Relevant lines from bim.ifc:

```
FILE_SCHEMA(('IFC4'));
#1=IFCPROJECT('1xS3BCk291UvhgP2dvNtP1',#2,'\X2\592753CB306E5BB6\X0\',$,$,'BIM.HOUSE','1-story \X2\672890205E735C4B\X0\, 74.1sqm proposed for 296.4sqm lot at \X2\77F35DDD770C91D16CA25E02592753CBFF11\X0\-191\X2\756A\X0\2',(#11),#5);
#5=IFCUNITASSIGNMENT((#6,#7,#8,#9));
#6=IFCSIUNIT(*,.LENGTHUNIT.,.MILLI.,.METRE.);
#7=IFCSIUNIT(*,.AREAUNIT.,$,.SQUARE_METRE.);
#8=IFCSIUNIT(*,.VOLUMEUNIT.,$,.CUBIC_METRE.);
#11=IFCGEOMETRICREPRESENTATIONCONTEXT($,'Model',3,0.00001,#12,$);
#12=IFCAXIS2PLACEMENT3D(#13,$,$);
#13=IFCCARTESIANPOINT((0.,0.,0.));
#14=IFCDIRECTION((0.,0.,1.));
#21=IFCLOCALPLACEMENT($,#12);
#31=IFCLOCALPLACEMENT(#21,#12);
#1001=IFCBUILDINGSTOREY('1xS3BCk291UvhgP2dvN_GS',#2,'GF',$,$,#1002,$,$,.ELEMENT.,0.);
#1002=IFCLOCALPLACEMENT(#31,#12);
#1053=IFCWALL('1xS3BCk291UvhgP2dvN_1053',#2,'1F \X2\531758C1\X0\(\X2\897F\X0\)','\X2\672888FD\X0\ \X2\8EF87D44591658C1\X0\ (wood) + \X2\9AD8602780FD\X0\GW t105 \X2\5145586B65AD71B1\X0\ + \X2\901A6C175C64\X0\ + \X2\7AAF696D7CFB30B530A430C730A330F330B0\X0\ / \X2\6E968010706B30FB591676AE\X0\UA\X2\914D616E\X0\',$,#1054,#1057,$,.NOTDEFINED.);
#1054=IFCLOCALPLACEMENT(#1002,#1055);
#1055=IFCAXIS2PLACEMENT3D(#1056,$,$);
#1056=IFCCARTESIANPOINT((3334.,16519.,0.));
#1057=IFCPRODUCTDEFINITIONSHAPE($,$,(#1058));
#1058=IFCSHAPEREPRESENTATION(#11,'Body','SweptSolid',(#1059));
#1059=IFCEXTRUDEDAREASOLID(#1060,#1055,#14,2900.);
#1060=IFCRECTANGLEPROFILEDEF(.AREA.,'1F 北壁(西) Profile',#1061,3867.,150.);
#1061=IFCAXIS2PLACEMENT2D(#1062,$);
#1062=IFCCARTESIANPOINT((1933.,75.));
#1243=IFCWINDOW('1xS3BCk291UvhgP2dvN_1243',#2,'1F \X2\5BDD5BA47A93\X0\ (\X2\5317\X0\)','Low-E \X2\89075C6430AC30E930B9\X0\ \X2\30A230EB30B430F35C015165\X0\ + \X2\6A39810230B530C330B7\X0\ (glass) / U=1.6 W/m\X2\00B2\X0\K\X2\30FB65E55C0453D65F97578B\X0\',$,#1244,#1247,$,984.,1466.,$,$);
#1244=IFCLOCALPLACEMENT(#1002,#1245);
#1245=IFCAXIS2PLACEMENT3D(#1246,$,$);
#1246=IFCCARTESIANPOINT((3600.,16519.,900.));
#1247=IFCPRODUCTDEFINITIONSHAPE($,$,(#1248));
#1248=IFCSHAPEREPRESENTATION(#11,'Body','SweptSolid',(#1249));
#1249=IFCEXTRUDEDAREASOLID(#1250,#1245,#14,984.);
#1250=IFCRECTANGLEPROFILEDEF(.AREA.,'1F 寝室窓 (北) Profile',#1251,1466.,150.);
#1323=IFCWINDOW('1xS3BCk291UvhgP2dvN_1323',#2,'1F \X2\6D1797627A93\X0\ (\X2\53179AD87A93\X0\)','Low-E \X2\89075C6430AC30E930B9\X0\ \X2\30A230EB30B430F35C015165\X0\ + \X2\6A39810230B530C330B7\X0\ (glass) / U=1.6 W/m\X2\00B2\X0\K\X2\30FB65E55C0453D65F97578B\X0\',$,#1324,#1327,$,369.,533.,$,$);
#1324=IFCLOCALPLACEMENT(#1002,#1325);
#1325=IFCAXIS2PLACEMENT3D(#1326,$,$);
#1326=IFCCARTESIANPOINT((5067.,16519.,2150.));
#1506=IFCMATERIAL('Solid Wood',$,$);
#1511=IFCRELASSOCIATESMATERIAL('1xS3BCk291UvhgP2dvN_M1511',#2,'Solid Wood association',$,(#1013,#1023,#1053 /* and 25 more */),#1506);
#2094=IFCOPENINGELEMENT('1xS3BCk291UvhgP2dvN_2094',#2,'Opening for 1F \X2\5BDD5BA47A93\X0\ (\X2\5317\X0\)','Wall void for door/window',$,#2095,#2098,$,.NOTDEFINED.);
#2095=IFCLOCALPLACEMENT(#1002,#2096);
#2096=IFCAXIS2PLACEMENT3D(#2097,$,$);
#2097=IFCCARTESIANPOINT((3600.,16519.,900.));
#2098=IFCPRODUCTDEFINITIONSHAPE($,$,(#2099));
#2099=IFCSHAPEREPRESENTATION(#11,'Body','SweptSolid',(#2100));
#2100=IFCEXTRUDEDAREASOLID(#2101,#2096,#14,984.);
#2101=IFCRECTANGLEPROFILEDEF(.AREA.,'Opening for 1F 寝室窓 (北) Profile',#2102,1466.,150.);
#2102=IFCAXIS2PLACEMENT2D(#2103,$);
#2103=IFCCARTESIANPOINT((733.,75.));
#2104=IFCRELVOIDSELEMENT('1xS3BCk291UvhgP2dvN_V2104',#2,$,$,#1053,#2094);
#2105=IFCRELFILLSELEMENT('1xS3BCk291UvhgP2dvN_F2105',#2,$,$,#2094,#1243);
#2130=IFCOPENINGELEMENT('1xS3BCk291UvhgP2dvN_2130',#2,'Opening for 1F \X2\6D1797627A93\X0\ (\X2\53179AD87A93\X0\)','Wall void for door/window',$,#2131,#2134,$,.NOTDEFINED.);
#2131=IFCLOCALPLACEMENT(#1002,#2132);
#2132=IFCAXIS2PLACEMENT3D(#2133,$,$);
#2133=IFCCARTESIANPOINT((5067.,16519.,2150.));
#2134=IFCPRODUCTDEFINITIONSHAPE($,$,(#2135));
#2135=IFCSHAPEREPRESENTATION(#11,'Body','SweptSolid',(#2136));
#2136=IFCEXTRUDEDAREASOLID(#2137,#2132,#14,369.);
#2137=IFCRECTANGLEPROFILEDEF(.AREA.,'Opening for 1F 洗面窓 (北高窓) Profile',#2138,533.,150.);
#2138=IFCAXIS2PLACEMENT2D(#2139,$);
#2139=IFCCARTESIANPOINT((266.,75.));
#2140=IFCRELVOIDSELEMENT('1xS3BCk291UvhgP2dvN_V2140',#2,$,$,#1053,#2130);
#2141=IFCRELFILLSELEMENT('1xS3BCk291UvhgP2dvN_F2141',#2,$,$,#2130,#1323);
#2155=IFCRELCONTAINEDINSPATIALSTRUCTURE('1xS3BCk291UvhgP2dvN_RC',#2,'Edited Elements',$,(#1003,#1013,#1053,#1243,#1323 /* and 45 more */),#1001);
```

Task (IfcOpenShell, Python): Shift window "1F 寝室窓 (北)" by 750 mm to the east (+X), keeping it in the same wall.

```python
import ifcopenshell
import ifcopenshell.api.geometry
import ifcopenshell.util.placement
import ifcopenshell.util.unit

model = ifcopenshell.open("bim.ifc")
unit_scale = ifcopenshell.util.unit.calculate_unit_scale(model)

window = model.by_guid("1xS3BCk291UvhgP2dvN_1243")
opening = window.FillsVoids[0].RelatingOpeningElement
wall = opening.VoidsElements[0].RelatingBuildingElement

wall_matrix = ifcopenshell.util.placement.get_local_placement(wall.ObjectPlacement)
shift = wall_matrix[:3, 0] * 0.75 / unit_scale
before = ifcopenshell.util.placement.get_local_placement(window.ObjectPlacement)[:3, 3].copy()

# The window is not placed relative to its opening, so move both.
for product in (opening, window):
    matrix = ifcopenshell.util.placement.get_local_placement(product.ObjectPlacement)
    matrix[:3, 3] += shift
    ifcopenshell.api.geometry.edit_object_placement(model, product=product, matrix=matrix, is_si=False)

after = ifcopenshell.util.placement.get_local_placement(window.ObjectPlacement)[:3, 3]
print("window moved by", (after - before).round(3) + 0.0)

model.write("bim_v2.ifc")
```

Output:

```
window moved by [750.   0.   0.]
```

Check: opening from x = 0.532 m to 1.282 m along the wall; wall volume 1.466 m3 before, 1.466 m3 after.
